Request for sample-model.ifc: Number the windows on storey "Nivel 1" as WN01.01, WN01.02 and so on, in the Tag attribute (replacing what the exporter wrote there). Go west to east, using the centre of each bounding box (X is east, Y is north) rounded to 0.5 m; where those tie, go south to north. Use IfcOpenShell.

First a look at what the model holds.

```python
import ifcopenshell
import ifcopenshell.util.element
import ifcopenshell.util.placement

model = ifcopenshell.open("sample-model.ifc")
print(model.schema)
storey = next(s for s in model.by_type("IfcBuildingStorey") if s.Name == "Nivel 1")
windows = [e for e in ifcopenshell.util.element.get_decomposition(storey) if e.is_a("IfcWindow")]
for e in sorted(windows, key=lambda e: e.id()):
    origin = ifcopenshell.util.placement.get_local_placement(e.ObjectPlacement)[:3, 3]
    print(e.id(), e.Tag, e.Name, origin.round(2) + 0.0, sep=" | ")
```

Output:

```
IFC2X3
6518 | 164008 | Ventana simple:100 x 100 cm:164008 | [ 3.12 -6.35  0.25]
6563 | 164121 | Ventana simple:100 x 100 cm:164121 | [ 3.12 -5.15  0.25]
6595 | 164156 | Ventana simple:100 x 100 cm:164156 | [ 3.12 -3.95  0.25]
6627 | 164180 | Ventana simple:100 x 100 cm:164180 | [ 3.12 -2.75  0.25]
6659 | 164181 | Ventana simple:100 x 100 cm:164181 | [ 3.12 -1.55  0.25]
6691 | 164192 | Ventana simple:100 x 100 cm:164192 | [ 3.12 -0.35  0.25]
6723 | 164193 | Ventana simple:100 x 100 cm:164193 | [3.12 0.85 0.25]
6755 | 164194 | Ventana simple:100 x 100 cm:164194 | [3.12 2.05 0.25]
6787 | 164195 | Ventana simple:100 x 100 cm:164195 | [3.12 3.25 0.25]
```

```python
import ifcopenshell
import ifcopenshell.geom
import ifcopenshell.util.element
import ifcopenshell.util.shape

model = ifcopenshell.open("sample-model.ifc")
settings = ifcopenshell.geom.settings()
settings.set("use-world-coords", True)


def centre(element):
    shape = ifcopenshell.geom.create_shape(settings, element)
    return ifcopenshell.util.shape.get_bbox_centroid(shape.geometry)


storey = next(s for s in model.by_type("IfcBuildingStorey") if s.Name == "Nivel 1")
windows = [e for e in ifcopenshell.util.element.get_decomposition(storey) if e.is_a("IfcWindow")]

# Insertion points can sit at a corner or the storey origin, so sort by the geometry (in metres).
centres = {e: centre(e) for e in windows}
windows.sort(key=lambda e: (round(centres[e][0] / 0.5), centres[e][1]))

for i, e in enumerate(windows, start=1):
    number = f"WN01.{i:02d}"
    e.Tag = number
    print(e.id(), number)

model.write("sample-model_updated.ifc")
```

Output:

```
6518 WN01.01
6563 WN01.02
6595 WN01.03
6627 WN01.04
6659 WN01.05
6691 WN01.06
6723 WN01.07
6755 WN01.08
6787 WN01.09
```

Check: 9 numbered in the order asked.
